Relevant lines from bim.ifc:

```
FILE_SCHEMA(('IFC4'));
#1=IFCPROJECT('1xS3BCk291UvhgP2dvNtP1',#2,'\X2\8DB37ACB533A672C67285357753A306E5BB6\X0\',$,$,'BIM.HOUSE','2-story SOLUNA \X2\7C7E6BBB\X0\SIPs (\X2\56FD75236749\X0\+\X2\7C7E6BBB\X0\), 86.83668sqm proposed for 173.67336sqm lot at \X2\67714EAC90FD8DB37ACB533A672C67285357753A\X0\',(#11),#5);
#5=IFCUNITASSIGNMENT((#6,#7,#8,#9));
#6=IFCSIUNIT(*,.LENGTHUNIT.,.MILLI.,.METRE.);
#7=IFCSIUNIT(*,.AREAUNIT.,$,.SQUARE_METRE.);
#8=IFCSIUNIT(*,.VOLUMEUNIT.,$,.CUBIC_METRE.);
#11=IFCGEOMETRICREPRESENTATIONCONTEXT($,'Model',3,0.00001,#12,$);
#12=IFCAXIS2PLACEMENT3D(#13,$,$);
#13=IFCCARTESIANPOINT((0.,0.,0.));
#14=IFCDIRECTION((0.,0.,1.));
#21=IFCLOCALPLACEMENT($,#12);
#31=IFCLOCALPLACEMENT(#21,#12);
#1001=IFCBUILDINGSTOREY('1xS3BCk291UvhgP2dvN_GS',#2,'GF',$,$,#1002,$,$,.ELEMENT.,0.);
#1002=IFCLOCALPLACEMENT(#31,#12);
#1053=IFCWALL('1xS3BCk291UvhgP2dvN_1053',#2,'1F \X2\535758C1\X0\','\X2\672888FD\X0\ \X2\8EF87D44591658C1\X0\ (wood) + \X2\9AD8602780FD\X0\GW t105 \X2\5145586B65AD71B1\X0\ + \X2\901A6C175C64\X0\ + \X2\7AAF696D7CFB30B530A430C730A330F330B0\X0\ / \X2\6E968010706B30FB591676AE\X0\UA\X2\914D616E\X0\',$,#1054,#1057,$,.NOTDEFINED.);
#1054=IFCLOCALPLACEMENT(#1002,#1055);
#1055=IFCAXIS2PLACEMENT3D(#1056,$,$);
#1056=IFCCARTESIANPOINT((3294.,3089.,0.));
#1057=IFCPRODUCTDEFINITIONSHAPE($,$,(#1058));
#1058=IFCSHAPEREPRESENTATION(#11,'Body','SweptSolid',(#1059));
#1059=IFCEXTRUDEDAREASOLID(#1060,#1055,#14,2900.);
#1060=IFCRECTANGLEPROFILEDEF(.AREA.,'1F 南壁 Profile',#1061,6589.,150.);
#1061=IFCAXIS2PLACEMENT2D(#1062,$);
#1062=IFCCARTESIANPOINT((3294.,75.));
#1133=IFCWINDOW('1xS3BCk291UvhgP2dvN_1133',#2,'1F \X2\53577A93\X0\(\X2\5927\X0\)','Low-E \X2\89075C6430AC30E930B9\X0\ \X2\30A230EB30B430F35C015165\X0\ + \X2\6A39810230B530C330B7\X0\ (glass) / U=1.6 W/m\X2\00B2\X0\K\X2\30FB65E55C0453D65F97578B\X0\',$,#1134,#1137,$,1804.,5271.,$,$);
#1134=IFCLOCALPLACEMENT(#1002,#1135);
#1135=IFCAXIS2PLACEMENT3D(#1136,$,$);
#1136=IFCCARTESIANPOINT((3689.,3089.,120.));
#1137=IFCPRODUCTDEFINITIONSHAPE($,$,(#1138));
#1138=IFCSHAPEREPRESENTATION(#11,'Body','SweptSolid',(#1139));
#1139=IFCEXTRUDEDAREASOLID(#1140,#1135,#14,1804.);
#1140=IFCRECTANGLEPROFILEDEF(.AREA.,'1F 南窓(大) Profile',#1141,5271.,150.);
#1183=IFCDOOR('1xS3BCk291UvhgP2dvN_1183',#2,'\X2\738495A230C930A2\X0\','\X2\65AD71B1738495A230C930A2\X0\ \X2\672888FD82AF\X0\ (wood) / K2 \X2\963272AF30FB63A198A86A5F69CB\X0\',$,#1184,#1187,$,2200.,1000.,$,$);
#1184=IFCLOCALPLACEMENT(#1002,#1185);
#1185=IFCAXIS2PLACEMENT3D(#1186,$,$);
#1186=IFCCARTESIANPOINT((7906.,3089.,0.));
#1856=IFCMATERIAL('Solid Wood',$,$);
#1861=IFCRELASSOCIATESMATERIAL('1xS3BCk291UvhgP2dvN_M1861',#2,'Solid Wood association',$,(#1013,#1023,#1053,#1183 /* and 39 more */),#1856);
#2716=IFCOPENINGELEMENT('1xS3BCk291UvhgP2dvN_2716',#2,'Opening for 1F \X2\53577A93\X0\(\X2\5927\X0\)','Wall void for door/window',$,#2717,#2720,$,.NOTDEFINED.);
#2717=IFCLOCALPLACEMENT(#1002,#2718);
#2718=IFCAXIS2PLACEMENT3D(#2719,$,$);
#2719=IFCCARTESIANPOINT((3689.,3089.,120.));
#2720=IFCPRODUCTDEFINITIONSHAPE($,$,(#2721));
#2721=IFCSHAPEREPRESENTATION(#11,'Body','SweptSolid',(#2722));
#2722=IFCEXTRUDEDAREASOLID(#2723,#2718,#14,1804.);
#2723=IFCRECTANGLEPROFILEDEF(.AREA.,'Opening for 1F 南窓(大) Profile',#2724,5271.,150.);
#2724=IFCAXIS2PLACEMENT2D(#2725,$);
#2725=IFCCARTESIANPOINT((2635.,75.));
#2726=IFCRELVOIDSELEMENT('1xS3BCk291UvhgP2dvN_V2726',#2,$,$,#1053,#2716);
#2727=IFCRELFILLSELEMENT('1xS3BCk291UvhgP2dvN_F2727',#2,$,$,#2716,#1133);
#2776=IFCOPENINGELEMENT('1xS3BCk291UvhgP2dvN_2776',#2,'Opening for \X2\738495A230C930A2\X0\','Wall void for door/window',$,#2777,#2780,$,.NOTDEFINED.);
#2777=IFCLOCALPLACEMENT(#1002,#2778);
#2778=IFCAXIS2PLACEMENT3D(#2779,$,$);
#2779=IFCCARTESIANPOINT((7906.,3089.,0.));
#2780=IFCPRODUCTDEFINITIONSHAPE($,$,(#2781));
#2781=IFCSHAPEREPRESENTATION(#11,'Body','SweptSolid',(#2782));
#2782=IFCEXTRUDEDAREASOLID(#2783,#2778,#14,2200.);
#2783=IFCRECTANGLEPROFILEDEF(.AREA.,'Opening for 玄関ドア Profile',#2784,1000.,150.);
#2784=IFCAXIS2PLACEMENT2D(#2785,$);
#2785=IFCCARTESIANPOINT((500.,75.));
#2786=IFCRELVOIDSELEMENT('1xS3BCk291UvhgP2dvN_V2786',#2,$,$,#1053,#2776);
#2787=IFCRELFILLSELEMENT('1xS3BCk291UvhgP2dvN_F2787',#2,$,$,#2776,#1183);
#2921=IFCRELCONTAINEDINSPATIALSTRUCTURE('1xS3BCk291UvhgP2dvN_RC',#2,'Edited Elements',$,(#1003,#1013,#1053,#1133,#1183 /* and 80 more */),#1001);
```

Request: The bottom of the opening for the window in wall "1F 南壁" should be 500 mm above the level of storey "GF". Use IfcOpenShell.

```python
import numpy as np
import ifcopenshell
import ifcopenshell.api.geometry
import ifcopenshell.geom
import ifcopenshell.util.element
import ifcopenshell.util.placement
import ifcopenshell.util.shape
import ifcopenshell.util.unit

model = ifcopenshell.open("bim.ifc")
unit_scale = ifcopenshell.util.unit.calculate_unit_scale(model)

window = model.by_guid("1xS3BCk291UvhgP2dvN_1133")
opening = window.FillsVoids[0].RelatingOpeningElement
storey = ifcopenshell.util.element.get_container(window, ifc_class="IfcBuildingStorey")
level = ifcopenshell.util.placement.get_local_placement(storey.ObjectPlacement)[2, 3]

# The opening's origin need not be at the sill, so measure its lowest point.
shape = ifcopenshell.geom.create_shape(ifcopenshell.geom.settings(), opening)
bottom = ifcopenshell.util.shape.get_shape_bottom_elevation(shape, shape.geometry) / unit_scale
dz = level + 500.0 - bottom

shift = np.array([0.0, 0.0, dz])
# The window is not placed relative to its opening, so move both.
for product in (opening, window):
    matrix = ifcopenshell.util.placement.get_local_placement(product.ObjectPlacement)
    matrix[:3, 3] += shift
    ifcopenshell.api.geometry.edit_object_placement(model, product=product, matrix=matrix, is_si=False)

print(f"moved by {dz * unit_scale:+.3f} m")

model.write("bim-out.ifc")
```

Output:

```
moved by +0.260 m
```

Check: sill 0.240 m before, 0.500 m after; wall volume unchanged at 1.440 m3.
